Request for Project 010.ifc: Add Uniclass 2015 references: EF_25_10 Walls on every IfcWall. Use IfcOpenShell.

First a look at what the model holds.

```python
import ifcopenshell

model = ifcopenshell.open("Project 010.ifc")
print(model.schema)
print("classifications:", [c.Name for c in model.by_type("IfcClassification")])
for ifc_class in ("IfcDoor", "IfcRoof", "IfcStair", "IfcWall", "IfcWindow"):
    print(ifc_class, len(model.by_type(ifc_class)))
```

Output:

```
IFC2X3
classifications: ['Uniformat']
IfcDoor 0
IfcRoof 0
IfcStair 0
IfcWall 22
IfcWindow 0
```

```python
import ifcopenshell
import ifcopenshell.api.classification

model = ifcopenshell.open("Project 010.ifc")

# IFC2X3 requires Source and Edition and has no link from the project to the system.
system = model.create_entity("IfcClassification", Source="NBS", Edition="2015", Name="Uniclass 2015")

codes = {
    "IfcWall": ("EF_25_10", "Walls"),
}
for ifc_class, (code, name) in codes.items():
    products = model.by_type(ifc_class)
    ifcopenshell.api.classification.add_reference(
        model, products=products, classification=system, identification=code, name=name
    )
    print(code, len(products))

model.write("Project 010_edited.ifc")
```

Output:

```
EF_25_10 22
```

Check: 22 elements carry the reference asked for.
